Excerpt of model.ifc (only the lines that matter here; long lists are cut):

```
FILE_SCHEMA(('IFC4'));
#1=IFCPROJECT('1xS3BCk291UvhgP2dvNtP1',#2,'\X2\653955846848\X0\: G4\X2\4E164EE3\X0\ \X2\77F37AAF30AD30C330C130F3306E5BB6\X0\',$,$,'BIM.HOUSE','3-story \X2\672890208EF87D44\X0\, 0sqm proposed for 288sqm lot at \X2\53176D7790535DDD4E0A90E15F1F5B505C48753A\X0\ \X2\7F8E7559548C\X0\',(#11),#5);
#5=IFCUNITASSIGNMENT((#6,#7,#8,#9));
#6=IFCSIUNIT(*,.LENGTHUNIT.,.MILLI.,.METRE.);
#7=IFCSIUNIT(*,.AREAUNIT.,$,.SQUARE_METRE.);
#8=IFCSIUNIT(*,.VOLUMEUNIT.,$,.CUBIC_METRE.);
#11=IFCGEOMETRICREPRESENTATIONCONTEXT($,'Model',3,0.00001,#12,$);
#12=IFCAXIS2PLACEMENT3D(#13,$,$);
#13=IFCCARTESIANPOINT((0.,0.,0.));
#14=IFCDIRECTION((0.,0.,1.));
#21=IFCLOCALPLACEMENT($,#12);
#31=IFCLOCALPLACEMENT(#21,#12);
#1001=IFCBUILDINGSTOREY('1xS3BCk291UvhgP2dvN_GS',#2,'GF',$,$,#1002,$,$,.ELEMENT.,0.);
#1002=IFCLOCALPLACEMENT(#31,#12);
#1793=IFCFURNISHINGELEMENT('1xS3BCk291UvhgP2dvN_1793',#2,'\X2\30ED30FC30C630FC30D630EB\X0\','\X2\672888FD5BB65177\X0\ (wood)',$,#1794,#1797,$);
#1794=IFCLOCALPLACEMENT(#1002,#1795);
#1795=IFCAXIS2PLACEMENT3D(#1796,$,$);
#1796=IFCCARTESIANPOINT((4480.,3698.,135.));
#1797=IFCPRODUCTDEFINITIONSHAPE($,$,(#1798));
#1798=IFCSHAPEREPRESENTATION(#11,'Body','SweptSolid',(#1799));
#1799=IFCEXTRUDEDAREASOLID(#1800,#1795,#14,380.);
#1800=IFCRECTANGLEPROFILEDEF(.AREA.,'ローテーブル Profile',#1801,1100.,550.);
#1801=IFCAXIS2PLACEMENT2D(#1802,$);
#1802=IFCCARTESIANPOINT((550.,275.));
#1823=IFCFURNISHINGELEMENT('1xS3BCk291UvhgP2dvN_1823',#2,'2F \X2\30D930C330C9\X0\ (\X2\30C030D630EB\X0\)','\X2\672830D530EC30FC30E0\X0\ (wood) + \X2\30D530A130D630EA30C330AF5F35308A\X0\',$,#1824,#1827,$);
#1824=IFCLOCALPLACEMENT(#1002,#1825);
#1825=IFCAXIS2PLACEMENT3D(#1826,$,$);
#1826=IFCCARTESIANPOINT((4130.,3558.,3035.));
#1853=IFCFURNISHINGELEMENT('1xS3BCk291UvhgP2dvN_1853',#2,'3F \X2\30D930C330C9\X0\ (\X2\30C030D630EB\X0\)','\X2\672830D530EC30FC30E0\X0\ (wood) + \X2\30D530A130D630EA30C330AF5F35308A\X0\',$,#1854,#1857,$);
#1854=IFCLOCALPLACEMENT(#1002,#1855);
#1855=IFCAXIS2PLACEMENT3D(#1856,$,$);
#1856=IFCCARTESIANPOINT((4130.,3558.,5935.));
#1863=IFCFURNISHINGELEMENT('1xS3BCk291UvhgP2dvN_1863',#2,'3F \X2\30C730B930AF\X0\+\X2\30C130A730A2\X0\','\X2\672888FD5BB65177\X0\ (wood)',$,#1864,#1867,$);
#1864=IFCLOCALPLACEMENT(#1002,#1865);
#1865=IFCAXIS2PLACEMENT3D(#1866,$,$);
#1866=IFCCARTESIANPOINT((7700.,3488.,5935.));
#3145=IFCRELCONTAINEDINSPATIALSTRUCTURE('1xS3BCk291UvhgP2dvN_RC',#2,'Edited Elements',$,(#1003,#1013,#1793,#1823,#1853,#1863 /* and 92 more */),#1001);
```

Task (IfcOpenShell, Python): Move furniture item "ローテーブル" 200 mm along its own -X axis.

```python
import ifcopenshell
import ifcopenshell.api.geometry
import ifcopenshell.util.placement
import ifcopenshell.util.unit

model = ifcopenshell.open("model.ifc")
unit_scale = ifcopenshell.util.unit.calculate_unit_scale(model)

item = model.by_guid("1xS3BCk291UvhgP2dvN_1793")
matrix = ifcopenshell.util.placement.get_local_placement(item.ObjectPlacement)
matrix[:3, 3] -= matrix[:3, 0] * 0.2 / unit_scale
ifcopenshell.api.geometry.edit_object_placement(model, product=item, matrix=matrix, is_si=False)

print(ifcopenshell.util.placement.get_local_placement(item.ObjectPlacement).round(3) + 0.0)

model.write("model_edited.ifc")
```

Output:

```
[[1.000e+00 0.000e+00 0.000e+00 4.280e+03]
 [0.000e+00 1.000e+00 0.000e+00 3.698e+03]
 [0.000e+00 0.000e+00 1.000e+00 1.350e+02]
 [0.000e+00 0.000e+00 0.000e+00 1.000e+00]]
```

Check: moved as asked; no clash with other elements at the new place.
